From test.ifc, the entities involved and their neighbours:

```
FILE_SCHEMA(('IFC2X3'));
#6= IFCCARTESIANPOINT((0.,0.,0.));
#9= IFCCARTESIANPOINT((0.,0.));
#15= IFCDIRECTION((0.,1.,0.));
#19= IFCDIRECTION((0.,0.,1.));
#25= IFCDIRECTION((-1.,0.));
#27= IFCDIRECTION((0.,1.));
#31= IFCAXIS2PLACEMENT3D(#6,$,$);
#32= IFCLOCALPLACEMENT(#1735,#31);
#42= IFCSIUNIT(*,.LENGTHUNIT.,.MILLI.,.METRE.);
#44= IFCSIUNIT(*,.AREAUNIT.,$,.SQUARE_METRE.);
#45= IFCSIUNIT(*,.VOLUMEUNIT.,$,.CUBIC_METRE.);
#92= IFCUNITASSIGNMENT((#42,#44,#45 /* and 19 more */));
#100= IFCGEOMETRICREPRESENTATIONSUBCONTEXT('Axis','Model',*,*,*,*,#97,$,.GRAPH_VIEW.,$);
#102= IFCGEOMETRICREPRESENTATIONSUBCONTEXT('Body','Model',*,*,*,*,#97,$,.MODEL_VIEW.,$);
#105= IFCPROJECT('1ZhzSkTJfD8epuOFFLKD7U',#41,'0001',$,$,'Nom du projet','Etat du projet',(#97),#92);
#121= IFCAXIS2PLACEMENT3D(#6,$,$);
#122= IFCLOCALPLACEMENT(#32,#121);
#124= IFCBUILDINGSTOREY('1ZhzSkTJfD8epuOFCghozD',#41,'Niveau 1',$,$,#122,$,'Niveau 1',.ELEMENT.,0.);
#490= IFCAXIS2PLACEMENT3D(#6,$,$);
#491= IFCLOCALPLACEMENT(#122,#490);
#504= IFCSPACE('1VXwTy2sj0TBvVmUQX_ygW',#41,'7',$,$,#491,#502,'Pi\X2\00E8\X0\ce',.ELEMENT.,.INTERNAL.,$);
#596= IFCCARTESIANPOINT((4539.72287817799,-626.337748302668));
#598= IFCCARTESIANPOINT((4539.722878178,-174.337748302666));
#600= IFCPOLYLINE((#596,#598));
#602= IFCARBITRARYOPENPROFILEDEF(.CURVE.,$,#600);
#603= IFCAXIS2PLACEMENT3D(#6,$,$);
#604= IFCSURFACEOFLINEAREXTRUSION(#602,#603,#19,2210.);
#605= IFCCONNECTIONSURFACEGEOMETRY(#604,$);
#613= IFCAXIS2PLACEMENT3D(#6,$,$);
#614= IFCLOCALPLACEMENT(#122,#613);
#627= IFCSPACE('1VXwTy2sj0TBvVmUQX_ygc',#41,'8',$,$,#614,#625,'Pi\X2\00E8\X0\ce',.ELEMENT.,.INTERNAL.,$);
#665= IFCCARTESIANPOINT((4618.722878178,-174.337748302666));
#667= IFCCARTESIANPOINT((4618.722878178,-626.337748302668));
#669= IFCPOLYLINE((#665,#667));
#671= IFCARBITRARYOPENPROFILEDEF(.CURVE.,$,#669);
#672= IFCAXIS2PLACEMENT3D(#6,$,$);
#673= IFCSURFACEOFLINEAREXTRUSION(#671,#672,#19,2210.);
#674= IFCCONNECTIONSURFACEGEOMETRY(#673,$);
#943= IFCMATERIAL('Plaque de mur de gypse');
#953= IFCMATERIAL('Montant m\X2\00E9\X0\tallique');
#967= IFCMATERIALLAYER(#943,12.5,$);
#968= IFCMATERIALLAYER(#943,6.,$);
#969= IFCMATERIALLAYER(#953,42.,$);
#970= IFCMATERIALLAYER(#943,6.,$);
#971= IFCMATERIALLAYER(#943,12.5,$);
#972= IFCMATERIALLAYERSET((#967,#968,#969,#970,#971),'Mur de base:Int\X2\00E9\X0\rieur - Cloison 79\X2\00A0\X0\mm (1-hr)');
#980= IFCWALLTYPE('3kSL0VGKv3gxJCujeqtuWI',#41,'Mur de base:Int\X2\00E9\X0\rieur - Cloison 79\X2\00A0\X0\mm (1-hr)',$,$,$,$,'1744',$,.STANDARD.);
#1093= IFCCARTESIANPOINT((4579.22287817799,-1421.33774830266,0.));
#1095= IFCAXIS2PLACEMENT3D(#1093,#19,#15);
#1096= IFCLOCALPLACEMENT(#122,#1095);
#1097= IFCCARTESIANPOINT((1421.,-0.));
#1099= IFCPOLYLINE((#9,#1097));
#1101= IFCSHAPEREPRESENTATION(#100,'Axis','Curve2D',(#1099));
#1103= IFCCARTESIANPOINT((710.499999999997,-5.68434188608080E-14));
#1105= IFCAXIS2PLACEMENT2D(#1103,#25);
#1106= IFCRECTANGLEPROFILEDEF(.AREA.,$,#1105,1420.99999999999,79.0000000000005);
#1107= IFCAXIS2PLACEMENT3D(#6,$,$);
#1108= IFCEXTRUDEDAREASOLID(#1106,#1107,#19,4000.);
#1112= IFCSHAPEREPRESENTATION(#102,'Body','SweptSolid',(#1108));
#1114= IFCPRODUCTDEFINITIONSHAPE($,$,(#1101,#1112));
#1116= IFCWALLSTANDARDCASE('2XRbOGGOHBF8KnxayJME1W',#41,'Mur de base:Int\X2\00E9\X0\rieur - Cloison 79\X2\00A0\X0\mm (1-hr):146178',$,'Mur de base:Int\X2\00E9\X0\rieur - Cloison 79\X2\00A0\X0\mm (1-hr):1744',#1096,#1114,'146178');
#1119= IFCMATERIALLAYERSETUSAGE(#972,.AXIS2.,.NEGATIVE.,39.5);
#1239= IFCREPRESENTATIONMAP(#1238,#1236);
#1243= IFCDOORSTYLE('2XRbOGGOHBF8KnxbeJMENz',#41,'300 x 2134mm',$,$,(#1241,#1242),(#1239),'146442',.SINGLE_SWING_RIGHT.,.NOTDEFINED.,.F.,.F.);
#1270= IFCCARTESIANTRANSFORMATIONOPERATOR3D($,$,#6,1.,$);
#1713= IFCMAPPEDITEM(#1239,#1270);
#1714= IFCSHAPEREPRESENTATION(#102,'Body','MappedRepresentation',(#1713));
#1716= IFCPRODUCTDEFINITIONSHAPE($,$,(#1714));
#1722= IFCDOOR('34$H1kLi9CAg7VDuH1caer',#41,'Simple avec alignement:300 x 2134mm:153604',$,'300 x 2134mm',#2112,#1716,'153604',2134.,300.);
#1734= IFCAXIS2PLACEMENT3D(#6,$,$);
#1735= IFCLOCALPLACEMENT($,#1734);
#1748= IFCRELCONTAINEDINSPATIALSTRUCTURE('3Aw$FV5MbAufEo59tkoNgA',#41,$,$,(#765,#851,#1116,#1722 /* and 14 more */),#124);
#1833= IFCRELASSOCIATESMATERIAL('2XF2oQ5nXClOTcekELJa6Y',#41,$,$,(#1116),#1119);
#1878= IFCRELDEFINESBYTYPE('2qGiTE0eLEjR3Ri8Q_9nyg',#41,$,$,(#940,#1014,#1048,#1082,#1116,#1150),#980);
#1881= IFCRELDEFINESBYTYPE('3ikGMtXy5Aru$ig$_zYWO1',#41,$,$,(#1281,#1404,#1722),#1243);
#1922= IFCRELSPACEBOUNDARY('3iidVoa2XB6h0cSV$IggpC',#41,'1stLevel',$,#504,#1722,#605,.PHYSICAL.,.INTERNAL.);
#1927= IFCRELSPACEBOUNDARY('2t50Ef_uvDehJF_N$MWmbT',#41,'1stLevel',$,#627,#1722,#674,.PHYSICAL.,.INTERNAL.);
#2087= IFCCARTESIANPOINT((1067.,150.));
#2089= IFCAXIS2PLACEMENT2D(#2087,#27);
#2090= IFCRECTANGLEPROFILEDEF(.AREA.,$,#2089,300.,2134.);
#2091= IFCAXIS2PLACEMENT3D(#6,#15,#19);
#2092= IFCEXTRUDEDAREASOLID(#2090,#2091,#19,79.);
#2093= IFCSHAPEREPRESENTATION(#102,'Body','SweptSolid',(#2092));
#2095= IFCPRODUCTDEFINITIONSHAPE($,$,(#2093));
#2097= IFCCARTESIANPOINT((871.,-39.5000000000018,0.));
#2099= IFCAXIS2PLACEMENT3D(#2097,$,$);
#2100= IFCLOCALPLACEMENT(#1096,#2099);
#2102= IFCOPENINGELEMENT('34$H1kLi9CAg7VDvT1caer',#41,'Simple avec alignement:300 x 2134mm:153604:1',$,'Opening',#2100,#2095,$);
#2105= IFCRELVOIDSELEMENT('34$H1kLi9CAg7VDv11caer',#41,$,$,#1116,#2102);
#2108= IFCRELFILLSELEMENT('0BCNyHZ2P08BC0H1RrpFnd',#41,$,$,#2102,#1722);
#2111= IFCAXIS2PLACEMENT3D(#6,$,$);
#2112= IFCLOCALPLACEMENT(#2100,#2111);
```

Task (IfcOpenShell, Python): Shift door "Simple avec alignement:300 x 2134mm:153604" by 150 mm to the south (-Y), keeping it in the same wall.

```python
import numpy as np
import ifcopenshell
import ifcopenshell.api.geometry
import ifcopenshell.util.placement
import ifcopenshell.util.unit

model = ifcopenshell.open("test.ifc")
unit_scale = ifcopenshell.util.unit.calculate_unit_scale(model)

door = model.by_id(1722)
opening = door.FillsVoids[0].RelatingOpeningElement
wall = opening.VoidsElements[0].RelatingBuildingElement

wall_matrix = ifcopenshell.util.placement.get_local_placement(wall.ObjectPlacement)
shift = wall_matrix[:3, 0] * -0.15 / unit_scale
before = ifcopenshell.util.placement.get_local_placement(door.ObjectPlacement)[:3, 3].copy()

# The door is placed relative to its opening, so it follows when the opening moves.
matrix = ifcopenshell.util.placement.get_local_placement(opening.ObjectPlacement)
matrix[:3, 3] += shift
ifcopenshell.api.geometry.edit_object_placement(
    model, product=opening, matrix=matrix, is_si=False, should_transform_children=True
)

# Space boundary surfaces are stored in each space's coordinates; move them too.
for rel in door.ProvidesBoundaries:
    if not rel.ConnectionGeometry:
        continue
    surface = rel.ConnectionGeometry.SurfaceOnRelatingElement
    space_matrix = ifcopenshell.util.placement.get_local_placement(rel.RelatingSpace.ObjectPlacement)
    point = np.array(surface.Position.Location.Coordinates) + space_matrix[:3, :3].T @ shift
    surface.Position = model.createIfcAxis2Placement3D(
        model.createIfcCartesianPoint(point.tolist()), surface.Position.Axis, surface.Position.RefDirection
    )

after = ifcopenshell.util.placement.get_local_placement(door.ObjectPlacement)[:3, 3]
print("door moved by", (after - before).round(3) + 0.0)

model.write("test_v2.ifc")
```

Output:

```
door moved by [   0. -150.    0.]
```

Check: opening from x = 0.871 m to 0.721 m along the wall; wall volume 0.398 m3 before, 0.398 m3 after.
